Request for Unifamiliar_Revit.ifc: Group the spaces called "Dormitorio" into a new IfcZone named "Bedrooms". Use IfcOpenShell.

First a look at what the model holds.

```python
import ifcopenshell

model = ifcopenshell.open("Unifamiliar_Revit.ifc")
print(model.schema)
seen = {}
for space in model.by_type("IfcSpace"):
    seen[space.LongName] = seen.get(space.LongName, 0) + 1
for name, count in sorted(seen.items(), key=str):
    print(count, "x", name)
print("zones:", [z.Name for z in model.by_type("IfcZone")][:20])
```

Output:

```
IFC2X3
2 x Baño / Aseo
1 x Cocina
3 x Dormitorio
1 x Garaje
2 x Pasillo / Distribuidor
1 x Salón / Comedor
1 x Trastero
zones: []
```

```python
import ifcopenshell
import ifcopenshell.api.group
import ifcopenshell.api.root

model = ifcopenshell.open("Unifamiliar_Revit.ifc")

names = {"Dormitorio"}
spaces = [s for s in model.by_type("IfcSpace") if s.LongName in names]

zone = ifcopenshell.api.root.create_entity(model, ifc_class="IfcZone", name="Bedrooms")
ifcopenshell.api.group.assign_group(model, products=spaces, group=zone)
print(len(spaces), "spaces in", zone.Name)

model.write("Unifamiliar_Revit_v2.ifc")
```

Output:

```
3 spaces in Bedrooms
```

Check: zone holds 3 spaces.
